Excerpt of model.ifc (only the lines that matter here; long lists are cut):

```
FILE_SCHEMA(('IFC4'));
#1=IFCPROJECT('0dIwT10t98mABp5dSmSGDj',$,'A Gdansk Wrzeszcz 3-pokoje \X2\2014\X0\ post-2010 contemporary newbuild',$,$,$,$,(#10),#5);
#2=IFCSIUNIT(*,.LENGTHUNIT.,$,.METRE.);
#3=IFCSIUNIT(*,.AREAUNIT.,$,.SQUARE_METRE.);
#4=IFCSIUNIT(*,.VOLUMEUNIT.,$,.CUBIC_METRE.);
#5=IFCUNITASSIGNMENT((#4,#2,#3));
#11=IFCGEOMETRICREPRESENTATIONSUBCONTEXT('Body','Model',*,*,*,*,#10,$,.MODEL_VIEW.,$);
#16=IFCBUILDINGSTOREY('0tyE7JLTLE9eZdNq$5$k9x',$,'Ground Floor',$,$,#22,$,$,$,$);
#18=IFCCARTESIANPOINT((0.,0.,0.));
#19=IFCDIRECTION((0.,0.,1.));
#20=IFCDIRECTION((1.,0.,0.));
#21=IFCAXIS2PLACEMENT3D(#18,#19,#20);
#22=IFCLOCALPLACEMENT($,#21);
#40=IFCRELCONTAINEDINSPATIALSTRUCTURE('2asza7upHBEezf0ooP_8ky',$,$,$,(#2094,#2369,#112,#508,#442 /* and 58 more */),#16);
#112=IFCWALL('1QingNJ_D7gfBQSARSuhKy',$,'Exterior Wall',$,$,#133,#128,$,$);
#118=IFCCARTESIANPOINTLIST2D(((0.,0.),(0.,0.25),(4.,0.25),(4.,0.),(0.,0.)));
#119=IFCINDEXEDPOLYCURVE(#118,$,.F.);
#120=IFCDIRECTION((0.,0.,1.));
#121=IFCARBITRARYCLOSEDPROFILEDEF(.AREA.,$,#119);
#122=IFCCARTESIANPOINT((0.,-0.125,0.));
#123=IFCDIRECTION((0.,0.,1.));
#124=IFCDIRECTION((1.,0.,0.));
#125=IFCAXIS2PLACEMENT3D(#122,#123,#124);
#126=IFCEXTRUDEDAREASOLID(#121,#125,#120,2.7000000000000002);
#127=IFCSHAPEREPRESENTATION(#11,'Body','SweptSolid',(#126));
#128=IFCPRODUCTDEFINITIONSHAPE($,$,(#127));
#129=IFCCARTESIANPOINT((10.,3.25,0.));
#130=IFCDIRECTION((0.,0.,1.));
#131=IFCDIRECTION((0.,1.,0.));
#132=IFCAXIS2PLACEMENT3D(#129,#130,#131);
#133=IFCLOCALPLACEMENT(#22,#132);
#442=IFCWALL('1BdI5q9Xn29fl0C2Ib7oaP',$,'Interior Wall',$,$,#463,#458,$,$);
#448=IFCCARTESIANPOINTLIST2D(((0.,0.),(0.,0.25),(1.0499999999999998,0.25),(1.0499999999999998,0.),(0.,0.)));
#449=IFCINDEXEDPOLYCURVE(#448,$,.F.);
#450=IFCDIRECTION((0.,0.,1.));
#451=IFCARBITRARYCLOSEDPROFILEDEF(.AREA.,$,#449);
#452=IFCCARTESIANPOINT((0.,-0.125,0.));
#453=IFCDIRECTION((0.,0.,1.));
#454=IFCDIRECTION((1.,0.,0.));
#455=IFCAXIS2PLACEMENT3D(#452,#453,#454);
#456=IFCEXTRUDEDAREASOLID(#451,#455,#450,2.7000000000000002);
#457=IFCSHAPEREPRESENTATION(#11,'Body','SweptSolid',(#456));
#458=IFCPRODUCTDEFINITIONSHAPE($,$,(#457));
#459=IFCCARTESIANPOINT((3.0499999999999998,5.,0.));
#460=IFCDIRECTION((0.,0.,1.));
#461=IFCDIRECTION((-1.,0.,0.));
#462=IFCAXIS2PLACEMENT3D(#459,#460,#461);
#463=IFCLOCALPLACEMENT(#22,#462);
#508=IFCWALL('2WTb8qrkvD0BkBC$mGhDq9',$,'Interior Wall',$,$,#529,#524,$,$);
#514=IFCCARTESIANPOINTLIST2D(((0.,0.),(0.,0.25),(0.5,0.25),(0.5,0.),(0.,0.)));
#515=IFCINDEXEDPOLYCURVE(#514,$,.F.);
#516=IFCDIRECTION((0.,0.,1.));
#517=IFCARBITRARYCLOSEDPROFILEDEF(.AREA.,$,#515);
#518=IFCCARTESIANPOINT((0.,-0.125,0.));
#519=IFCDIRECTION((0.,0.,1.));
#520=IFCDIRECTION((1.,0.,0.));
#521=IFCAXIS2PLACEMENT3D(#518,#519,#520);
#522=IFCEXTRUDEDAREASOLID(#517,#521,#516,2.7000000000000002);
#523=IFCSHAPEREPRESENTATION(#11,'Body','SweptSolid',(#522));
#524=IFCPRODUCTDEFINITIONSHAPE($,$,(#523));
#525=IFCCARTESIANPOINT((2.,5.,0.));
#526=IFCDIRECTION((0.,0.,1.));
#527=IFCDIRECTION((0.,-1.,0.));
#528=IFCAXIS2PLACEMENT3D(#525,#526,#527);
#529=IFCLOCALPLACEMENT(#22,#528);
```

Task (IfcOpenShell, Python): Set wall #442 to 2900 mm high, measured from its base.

```python
import ifcopenshell
import ifcopenshell.geom
import ifcopenshell.util.representation
import ifcopenshell.util.shape
import ifcopenshell.util.unit

model = ifcopenshell.open("model.ifc")
unit_scale = ifcopenshell.util.unit.calculate_unit_scale(model)
settings = ifcopenshell.geom.settings()


def volume(element):
    """Net volume in cubic metres, openings subtracted."""
    shape = ifcopenshell.geom.create_shape(settings, element)
    return ifcopenshell.util.shape.get_volume(shape.geometry)


wall = model.by_id(442)
before = volume(wall)

body = ifcopenshell.util.representation.get_representation(wall, "Model", "Body")
solid = body.Items[0]
old_height = solid.Depth
solid.Depth = 2.9 / unit_scale
after = volume(wall)

print(f"height {old_height:g} -> {solid.Depth:g}, volume {before:.3f} -> {after:.3f} m3")

model.write("model_updated.ifc")
```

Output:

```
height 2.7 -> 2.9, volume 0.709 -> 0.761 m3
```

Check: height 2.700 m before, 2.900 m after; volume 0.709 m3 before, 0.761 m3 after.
